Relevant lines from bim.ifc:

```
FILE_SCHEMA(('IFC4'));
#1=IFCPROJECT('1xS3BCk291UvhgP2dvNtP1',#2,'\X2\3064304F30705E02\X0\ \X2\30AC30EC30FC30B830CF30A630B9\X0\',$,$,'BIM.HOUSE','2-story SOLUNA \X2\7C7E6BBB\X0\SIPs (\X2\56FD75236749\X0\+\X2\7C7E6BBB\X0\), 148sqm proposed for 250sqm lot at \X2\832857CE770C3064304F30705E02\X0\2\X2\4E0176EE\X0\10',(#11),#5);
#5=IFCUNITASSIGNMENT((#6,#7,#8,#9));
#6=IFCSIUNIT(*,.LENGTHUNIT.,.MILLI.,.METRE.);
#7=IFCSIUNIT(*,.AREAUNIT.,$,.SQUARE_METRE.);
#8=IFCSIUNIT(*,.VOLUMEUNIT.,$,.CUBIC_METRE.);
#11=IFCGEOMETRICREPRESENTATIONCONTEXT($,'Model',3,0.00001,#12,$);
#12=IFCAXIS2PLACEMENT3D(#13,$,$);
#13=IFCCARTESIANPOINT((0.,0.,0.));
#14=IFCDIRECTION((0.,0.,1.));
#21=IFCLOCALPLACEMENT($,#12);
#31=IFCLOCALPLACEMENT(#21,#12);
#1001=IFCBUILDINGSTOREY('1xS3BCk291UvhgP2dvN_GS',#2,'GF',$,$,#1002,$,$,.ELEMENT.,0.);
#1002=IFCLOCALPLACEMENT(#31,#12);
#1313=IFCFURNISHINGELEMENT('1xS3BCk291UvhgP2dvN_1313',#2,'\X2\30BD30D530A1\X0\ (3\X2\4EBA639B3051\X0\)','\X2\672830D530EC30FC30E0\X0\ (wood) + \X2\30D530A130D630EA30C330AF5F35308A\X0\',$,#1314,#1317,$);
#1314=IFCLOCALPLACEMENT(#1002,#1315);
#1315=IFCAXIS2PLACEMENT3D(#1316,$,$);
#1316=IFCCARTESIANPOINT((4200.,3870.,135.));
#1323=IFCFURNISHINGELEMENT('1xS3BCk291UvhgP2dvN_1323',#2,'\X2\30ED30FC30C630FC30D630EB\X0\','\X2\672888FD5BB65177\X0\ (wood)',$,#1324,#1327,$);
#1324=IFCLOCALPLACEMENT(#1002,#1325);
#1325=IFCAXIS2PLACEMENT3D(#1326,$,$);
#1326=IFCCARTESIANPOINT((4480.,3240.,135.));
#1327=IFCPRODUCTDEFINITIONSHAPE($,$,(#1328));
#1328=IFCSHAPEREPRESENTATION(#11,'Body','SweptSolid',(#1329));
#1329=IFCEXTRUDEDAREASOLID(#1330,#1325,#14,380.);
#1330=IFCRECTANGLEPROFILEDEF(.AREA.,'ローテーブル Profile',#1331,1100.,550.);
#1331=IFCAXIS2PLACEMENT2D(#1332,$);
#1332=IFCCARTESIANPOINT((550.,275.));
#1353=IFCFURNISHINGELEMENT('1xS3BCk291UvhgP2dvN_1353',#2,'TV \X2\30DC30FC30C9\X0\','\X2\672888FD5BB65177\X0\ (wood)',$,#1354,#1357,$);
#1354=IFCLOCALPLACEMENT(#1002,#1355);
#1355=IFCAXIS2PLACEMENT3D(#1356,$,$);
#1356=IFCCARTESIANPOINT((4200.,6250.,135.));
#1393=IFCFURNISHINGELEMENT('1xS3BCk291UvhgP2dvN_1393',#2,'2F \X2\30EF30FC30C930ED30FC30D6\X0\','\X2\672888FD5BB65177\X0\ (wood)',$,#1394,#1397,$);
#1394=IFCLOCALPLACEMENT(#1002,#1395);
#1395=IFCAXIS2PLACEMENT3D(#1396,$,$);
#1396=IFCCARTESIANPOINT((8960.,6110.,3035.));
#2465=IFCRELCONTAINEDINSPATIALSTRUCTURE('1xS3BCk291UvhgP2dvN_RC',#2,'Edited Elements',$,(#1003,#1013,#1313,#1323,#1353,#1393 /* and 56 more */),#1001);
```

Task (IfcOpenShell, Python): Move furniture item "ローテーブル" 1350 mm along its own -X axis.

```python
import ifcopenshell
import ifcopenshell.api.geometry
import ifcopenshell.util.placement

model = ifcopenshell.open("bim.ifc")

item = model.by_id(1323)
matrix = ifcopenshell.util.placement.get_local_placement(item.ObjectPlacement)
matrix[:3, 3] -= matrix[:3, 0] * 1350.0
ifcopenshell.api.geometry.edit_object_placement(model, product=item, matrix=matrix, is_si=False)

print(ifcopenshell.util.placement.get_local_placement(item.ObjectPlacement).round(3) + 0.0)

model.write("bim-out.ifc")
```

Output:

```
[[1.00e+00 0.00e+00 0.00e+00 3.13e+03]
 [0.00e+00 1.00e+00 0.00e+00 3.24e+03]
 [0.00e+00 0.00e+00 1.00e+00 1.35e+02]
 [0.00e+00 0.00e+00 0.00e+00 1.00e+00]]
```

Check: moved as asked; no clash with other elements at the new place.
